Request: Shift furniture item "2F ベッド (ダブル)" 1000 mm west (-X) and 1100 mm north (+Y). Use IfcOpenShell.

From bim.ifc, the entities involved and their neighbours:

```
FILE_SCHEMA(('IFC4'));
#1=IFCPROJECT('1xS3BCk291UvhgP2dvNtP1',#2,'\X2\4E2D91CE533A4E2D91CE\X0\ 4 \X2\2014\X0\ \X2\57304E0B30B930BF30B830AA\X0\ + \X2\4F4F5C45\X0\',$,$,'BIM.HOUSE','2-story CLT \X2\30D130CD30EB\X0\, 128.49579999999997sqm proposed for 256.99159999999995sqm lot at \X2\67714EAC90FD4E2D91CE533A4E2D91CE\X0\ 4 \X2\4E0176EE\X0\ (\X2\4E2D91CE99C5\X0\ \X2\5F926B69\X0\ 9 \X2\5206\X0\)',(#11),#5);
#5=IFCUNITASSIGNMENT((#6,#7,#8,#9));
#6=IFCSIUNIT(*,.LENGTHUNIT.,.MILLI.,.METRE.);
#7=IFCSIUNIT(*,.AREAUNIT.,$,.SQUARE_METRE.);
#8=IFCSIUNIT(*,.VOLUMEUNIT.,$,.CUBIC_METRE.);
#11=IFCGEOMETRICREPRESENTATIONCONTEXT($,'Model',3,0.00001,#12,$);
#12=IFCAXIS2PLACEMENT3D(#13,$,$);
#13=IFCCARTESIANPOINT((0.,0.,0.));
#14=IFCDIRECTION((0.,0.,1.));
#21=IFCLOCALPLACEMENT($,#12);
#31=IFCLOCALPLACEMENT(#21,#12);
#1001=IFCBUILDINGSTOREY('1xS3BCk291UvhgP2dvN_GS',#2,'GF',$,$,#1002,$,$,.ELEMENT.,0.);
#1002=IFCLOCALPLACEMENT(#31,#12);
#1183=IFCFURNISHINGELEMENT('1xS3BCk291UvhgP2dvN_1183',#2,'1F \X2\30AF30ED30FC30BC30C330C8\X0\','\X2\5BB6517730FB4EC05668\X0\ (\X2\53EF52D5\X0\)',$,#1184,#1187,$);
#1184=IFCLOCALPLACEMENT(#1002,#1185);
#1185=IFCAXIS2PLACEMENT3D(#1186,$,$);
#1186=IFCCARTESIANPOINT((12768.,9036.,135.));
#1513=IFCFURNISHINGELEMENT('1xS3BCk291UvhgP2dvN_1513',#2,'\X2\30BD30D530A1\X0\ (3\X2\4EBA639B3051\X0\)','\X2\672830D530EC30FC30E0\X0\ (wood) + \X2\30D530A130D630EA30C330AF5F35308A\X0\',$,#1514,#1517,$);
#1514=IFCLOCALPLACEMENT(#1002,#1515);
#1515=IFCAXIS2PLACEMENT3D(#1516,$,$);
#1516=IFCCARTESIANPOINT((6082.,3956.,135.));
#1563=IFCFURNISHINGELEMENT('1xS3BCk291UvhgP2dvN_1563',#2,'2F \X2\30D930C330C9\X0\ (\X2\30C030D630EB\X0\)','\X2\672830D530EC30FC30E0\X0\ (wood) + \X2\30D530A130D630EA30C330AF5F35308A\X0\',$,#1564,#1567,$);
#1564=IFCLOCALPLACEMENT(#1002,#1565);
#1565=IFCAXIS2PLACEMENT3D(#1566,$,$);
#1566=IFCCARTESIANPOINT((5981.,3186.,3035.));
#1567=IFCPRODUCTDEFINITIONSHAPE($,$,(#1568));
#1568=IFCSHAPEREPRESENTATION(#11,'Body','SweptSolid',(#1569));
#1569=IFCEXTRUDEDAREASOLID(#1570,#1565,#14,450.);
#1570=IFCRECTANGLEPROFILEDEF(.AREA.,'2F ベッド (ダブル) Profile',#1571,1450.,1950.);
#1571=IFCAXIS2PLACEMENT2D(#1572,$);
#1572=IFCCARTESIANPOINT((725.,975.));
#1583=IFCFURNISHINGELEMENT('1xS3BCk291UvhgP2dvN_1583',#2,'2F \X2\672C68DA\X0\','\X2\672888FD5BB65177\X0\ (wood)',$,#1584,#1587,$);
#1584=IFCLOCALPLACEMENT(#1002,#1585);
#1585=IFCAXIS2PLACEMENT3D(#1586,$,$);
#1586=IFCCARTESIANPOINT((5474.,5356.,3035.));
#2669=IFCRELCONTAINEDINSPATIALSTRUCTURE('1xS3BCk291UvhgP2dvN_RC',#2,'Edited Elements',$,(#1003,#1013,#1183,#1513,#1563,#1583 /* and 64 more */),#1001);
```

```python
import ifcopenshell
import ifcopenshell.api.geometry
import ifcopenshell.util.placement
import ifcopenshell.util.unit

model = ifcopenshell.open("bim.ifc")
unit_scale = ifcopenshell.util.unit.calculate_unit_scale(model)

item = model.by_guid("1xS3BCk291UvhgP2dvN_1563")
matrix = ifcopenshell.util.placement.get_local_placement(item.ObjectPlacement)
matrix[0, 3] -= 1 / unit_scale
matrix[1, 3] += 1.1 / unit_scale
ifcopenshell.api.geometry.edit_object_placement(model, product=item, matrix=matrix, is_si=False)

print(ifcopenshell.util.placement.get_local_placement(item.ObjectPlacement).round(3) + 0.0)

model.write("bim_edited.ifc")
```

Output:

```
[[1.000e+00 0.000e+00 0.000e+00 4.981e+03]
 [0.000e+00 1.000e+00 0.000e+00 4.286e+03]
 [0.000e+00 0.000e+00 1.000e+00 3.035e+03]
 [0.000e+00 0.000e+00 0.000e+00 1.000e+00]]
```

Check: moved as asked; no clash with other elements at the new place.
